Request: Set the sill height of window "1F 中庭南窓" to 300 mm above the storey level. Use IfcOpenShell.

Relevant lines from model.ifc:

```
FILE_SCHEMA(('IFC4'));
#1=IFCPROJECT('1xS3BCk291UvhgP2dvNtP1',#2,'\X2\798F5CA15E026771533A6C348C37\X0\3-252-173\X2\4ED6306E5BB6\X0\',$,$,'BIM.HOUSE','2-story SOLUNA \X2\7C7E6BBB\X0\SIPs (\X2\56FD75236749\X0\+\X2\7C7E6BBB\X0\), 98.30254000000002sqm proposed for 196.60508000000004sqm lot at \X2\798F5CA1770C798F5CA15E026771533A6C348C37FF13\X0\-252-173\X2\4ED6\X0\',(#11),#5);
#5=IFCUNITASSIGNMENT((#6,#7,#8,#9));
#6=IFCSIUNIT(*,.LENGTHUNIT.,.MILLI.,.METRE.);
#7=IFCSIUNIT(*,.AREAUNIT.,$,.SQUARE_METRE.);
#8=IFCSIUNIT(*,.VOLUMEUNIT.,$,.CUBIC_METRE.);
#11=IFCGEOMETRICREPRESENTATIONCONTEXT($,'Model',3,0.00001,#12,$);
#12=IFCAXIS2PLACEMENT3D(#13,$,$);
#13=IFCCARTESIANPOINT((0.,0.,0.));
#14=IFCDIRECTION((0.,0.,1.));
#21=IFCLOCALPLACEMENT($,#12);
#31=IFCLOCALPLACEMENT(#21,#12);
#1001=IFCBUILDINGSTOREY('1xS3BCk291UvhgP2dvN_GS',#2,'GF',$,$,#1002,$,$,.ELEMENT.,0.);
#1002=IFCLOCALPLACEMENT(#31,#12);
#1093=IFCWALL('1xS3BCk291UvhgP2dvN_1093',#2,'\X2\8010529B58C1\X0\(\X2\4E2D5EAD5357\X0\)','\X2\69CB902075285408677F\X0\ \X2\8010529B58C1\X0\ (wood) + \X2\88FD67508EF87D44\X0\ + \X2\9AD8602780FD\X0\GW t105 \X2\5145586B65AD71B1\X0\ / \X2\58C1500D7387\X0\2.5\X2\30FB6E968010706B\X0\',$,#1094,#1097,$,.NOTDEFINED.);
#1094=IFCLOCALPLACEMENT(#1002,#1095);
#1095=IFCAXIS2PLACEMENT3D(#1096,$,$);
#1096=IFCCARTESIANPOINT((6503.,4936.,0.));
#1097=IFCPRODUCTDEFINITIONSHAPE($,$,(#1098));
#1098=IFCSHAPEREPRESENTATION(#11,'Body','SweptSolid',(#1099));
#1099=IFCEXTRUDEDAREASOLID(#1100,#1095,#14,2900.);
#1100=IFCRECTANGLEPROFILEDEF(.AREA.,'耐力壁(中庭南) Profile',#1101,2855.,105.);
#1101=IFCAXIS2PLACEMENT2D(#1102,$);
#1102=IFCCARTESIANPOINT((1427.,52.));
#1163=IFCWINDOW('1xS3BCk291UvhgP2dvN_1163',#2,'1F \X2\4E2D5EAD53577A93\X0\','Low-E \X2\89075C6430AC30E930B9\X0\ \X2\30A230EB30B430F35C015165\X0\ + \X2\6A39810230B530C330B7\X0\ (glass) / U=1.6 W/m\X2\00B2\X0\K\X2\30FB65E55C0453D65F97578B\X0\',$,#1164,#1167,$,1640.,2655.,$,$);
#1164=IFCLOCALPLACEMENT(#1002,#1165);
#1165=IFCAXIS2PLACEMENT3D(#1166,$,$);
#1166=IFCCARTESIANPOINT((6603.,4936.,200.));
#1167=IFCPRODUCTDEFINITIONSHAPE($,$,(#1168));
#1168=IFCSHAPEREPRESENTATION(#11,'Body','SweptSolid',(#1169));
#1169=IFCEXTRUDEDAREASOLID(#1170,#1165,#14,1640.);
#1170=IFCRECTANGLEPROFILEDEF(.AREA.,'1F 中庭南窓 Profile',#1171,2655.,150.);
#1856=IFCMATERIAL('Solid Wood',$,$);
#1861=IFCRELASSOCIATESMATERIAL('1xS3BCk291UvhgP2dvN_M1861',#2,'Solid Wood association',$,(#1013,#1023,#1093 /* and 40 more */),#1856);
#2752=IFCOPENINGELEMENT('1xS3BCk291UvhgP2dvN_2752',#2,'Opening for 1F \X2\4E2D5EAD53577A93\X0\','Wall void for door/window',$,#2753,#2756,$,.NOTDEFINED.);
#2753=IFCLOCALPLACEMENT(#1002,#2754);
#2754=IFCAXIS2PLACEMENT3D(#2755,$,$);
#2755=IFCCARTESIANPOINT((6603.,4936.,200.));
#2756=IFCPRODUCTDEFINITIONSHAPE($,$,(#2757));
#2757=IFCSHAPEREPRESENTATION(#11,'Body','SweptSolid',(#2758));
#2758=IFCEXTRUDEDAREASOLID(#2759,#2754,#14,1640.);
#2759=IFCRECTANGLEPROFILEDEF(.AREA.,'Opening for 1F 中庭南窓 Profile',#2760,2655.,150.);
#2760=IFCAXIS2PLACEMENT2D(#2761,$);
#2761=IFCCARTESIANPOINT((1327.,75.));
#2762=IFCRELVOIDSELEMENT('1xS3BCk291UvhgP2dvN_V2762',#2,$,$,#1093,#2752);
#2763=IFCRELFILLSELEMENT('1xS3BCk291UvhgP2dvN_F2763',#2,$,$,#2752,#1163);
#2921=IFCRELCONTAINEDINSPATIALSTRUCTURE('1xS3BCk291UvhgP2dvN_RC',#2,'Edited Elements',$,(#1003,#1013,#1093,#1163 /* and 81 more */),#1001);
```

```python
import numpy as np
import ifcopenshell
import ifcopenshell.api.geometry
import ifcopenshell.geom
import ifcopenshell.util.element
import ifcopenshell.util.placement
import ifcopenshell.util.shape
import ifcopenshell.util.unit

model = ifcopenshell.open("model.ifc")
unit_scale = ifcopenshell.util.unit.calculate_unit_scale(model)

window = model.by_guid("1xS3BCk291UvhgP2dvN_1163")
opening = window.FillsVoids[0].RelatingOpeningElement
storey = ifcopenshell.util.element.get_container(window, ifc_class="IfcBuildingStorey")
level = ifcopenshell.util.placement.get_local_placement(storey.ObjectPlacement)[2, 3]

# The opening's origin need not be at the sill, so measure its lowest point.
shape = ifcopenshell.geom.create_shape(ifcopenshell.geom.settings(), opening)
bottom = ifcopenshell.util.shape.get_shape_bottom_elevation(shape, shape.geometry) / unit_scale
dz = level + 300.0 - bottom

shift = np.array([0.0, 0.0, dz])
# The window is not placed relative to its opening, so move both.
for product in (opening, window):
    matrix = ifcopenshell.util.placement.get_local_placement(product.ObjectPlacement)
    matrix[:3, 3] += shift
    ifcopenshell.api.geometry.edit_object_placement(model, product=product, matrix=matrix, is_si=False)

print(f"moved by {dz * unit_scale:+.3f} m")

model.write("model_updated.ifc")
```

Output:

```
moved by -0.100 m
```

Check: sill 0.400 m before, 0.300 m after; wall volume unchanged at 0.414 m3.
